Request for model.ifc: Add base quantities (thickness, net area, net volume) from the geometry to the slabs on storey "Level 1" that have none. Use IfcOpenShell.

First a look at what the model holds.

```python
import ifcopenshell
import ifcopenshell.util.element
import ifcopenshell.util.unit

model = ifcopenshell.open("model.ifc")
print(model.schema)
for unit_type in ("LENGTHUNIT", "AREAUNIT", "VOLUMEUNIT"):
    print(unit_type, ifcopenshell.util.unit.calculate_unit_scale(model, unit_type))
storey = next(s for s in model.by_type("IfcBuildingStorey") if s.Name == "Level 1")
slabs = [e for e in ifcopenshell.util.element.get_decomposition(storey) if e.is_a("IfcSlab")]
for e in sorted(slabs, key=lambda e: e.id()):
    print(e.id(), e.is_a(), e.Name, list(ifcopenshell.util.element.get_psets(e, qtos_only=True)), sep=" | ")
```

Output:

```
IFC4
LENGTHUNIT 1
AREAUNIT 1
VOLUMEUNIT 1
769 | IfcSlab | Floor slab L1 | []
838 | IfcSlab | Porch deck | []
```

```python
import ifcopenshell
import ifcopenshell.api.pset
import ifcopenshell.geom
import ifcopenshell.util.element
import ifcopenshell.util.shape
import ifcopenshell.util.unit

model = ifcopenshell.open("model.ifc")
unit_scale = ifcopenshell.util.unit.calculate_unit_scale(model)
area_scale = ifcopenshell.util.unit.calculate_unit_scale(model, "AREAUNIT")
volume_scale = ifcopenshell.util.unit.calculate_unit_scale(model, "VOLUMEUNIT")
settings = ifcopenshell.geom.settings()

storey = next(s for s in model.by_type("IfcBuildingStorey") if s.Name == "Level 1")
slabs = [e for e in ifcopenshell.util.element.get_decomposition(storey) if e.is_a("IfcSlab")]

for e in sorted(slabs, key=lambda e: e.id()):
    if ifcopenshell.util.element.get_psets(e, qtos_only=True, should_inherit=False):
        continue
    # Geometry comes back in metres, in the element's own axes.
    shape = ifcopenshell.geom.create_shape(settings, e)
    values = {
        "Width": ifcopenshell.util.shape.get_z(shape.geometry) / unit_scale,
        "NetArea": ifcopenshell.util.shape.get_footprint_area(shape.geometry) / area_scale,
        "NetVolume": ifcopenshell.util.shape.get_volume(shape.geometry) / volume_scale,
    }
    qto = ifcopenshell.api.pset.add_qto(model, product=e, name="Qto_SlabBaseQuantities")
    ifcopenshell.api.pset.edit_qto(model, qto=qto, properties=values)
    print(e.id(), {k: round(v, 3) for k, v in values.items()})

model.write("model-out.ifc")
```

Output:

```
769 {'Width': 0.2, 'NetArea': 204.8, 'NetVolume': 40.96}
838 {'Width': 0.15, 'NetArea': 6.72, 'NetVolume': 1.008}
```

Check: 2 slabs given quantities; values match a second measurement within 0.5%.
